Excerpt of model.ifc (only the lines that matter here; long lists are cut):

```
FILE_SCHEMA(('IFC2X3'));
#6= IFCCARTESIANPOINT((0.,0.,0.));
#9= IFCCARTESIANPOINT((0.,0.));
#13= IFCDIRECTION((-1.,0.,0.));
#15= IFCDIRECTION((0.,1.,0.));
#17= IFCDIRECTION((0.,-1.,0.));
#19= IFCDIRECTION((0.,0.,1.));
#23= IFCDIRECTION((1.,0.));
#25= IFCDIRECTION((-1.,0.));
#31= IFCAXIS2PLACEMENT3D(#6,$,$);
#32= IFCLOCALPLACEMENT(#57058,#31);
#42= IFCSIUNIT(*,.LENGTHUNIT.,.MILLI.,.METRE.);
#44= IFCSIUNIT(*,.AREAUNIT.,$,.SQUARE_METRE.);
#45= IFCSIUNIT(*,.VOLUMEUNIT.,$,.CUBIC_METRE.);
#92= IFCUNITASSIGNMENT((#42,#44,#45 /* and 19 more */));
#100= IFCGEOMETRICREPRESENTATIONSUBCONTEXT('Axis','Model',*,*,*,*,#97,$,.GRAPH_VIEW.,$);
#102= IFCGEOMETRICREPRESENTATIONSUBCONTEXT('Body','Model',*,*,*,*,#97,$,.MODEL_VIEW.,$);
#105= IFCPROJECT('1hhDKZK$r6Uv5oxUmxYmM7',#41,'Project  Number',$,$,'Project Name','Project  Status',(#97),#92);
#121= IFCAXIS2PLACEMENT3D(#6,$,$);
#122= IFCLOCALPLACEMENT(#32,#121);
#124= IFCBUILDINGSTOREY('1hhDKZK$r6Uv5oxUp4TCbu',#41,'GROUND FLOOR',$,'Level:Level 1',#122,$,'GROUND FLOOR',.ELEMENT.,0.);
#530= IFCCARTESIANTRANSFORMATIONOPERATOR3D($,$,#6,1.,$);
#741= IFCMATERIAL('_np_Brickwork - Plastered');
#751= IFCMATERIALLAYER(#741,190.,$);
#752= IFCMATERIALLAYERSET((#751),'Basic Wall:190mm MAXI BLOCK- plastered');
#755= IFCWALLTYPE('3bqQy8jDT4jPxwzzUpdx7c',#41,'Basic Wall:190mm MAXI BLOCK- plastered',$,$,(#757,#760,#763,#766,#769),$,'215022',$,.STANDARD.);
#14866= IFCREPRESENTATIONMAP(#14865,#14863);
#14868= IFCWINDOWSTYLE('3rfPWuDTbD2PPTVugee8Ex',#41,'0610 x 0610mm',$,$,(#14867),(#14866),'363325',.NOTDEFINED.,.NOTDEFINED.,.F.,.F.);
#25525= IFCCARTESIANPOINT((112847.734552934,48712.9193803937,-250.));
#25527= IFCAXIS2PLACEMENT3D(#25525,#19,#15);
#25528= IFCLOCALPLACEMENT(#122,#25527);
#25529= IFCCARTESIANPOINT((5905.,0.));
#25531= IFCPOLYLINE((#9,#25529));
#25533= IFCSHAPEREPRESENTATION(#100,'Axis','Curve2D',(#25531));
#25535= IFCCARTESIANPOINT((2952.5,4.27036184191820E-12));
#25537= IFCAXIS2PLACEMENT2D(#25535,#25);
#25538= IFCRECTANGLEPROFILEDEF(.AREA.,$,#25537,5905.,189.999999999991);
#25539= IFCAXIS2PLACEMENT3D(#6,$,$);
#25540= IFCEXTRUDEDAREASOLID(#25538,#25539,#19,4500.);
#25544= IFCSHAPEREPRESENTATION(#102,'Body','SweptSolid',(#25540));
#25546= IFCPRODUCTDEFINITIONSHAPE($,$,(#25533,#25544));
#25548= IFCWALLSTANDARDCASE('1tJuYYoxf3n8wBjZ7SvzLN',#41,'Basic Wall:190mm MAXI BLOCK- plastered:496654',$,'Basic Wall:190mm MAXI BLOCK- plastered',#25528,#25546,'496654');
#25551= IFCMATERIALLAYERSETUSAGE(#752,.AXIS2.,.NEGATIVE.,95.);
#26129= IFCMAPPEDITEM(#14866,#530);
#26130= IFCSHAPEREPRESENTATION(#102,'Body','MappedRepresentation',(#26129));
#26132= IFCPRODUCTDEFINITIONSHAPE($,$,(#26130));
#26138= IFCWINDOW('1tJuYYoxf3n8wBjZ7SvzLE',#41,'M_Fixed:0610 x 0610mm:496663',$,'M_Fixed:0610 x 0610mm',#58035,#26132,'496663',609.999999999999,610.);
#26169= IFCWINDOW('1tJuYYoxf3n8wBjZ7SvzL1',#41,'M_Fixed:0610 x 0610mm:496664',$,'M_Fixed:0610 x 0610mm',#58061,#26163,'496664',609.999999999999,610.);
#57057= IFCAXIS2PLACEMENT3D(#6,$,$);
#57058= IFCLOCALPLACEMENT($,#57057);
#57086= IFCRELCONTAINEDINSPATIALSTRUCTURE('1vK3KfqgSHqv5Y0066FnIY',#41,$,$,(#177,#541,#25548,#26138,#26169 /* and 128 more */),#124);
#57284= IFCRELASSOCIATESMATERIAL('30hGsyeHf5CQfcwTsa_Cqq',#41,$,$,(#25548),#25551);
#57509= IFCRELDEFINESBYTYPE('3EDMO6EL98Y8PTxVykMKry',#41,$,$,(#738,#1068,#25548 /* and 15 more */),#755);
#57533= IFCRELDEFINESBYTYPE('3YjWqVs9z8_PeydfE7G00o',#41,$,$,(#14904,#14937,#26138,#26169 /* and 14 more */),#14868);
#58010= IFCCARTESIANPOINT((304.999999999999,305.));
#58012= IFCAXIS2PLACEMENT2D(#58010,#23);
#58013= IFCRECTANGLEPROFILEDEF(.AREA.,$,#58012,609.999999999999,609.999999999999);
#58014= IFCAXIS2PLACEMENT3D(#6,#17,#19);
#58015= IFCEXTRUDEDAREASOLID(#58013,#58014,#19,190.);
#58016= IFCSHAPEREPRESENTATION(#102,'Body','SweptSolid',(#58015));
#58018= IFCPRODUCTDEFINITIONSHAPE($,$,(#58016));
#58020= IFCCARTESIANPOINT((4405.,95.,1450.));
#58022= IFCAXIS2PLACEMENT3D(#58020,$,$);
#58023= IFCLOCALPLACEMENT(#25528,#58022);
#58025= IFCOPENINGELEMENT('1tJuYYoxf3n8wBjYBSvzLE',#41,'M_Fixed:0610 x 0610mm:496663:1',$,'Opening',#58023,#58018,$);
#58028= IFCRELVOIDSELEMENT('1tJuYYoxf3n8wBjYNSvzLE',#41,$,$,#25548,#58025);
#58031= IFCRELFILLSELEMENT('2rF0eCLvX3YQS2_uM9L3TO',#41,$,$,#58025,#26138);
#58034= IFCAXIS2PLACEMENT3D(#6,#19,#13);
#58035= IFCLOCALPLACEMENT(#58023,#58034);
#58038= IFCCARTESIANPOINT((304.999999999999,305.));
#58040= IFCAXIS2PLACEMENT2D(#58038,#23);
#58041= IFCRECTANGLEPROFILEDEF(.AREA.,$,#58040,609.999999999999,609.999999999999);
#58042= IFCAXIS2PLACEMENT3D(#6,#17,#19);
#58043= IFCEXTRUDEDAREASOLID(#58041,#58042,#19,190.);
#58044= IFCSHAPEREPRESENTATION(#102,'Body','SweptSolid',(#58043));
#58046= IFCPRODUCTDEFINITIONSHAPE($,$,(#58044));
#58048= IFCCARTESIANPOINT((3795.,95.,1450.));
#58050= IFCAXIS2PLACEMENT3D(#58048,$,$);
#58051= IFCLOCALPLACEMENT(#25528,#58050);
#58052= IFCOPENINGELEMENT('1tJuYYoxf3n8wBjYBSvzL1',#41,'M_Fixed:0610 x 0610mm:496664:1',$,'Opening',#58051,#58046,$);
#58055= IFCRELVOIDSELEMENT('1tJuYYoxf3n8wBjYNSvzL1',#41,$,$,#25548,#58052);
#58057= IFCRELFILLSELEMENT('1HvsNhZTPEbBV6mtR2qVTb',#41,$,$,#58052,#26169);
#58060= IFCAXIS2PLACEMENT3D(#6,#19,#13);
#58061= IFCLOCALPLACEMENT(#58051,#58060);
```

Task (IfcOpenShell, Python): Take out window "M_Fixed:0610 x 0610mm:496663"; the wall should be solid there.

```python
import ifcopenshell
import ifcopenshell.api.feature
import ifcopenshell.api.root
import ifcopenshell.geom
import ifcopenshell.util.shape

model = ifcopenshell.open("model.ifc")
settings = ifcopenshell.geom.settings()


def volume(element):
    """Net volume in cubic metres, openings subtracted."""
    shape = ifcopenshell.geom.create_shape(settings, element)
    return ifcopenshell.util.shape.get_volume(shape.geometry)


window = model.by_guid("1tJuYYoxf3n8wBjZ7SvzLE")
opening = window.FillsVoids[0].RelatingOpeningElement
wall = opening.VoidsElements[0].RelatingBuildingElement
before = volume(wall)

ifcopenshell.api.root.remove_product(model, product=window)
ifcopenshell.api.feature.remove_feature(model, feature=opening)

after = volume(wall)

print(f"wall volume {before:.3f} -> {after:.3f} m3")

model.write("model_edited.ifc")
```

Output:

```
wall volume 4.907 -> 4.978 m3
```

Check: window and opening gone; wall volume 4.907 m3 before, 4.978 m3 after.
